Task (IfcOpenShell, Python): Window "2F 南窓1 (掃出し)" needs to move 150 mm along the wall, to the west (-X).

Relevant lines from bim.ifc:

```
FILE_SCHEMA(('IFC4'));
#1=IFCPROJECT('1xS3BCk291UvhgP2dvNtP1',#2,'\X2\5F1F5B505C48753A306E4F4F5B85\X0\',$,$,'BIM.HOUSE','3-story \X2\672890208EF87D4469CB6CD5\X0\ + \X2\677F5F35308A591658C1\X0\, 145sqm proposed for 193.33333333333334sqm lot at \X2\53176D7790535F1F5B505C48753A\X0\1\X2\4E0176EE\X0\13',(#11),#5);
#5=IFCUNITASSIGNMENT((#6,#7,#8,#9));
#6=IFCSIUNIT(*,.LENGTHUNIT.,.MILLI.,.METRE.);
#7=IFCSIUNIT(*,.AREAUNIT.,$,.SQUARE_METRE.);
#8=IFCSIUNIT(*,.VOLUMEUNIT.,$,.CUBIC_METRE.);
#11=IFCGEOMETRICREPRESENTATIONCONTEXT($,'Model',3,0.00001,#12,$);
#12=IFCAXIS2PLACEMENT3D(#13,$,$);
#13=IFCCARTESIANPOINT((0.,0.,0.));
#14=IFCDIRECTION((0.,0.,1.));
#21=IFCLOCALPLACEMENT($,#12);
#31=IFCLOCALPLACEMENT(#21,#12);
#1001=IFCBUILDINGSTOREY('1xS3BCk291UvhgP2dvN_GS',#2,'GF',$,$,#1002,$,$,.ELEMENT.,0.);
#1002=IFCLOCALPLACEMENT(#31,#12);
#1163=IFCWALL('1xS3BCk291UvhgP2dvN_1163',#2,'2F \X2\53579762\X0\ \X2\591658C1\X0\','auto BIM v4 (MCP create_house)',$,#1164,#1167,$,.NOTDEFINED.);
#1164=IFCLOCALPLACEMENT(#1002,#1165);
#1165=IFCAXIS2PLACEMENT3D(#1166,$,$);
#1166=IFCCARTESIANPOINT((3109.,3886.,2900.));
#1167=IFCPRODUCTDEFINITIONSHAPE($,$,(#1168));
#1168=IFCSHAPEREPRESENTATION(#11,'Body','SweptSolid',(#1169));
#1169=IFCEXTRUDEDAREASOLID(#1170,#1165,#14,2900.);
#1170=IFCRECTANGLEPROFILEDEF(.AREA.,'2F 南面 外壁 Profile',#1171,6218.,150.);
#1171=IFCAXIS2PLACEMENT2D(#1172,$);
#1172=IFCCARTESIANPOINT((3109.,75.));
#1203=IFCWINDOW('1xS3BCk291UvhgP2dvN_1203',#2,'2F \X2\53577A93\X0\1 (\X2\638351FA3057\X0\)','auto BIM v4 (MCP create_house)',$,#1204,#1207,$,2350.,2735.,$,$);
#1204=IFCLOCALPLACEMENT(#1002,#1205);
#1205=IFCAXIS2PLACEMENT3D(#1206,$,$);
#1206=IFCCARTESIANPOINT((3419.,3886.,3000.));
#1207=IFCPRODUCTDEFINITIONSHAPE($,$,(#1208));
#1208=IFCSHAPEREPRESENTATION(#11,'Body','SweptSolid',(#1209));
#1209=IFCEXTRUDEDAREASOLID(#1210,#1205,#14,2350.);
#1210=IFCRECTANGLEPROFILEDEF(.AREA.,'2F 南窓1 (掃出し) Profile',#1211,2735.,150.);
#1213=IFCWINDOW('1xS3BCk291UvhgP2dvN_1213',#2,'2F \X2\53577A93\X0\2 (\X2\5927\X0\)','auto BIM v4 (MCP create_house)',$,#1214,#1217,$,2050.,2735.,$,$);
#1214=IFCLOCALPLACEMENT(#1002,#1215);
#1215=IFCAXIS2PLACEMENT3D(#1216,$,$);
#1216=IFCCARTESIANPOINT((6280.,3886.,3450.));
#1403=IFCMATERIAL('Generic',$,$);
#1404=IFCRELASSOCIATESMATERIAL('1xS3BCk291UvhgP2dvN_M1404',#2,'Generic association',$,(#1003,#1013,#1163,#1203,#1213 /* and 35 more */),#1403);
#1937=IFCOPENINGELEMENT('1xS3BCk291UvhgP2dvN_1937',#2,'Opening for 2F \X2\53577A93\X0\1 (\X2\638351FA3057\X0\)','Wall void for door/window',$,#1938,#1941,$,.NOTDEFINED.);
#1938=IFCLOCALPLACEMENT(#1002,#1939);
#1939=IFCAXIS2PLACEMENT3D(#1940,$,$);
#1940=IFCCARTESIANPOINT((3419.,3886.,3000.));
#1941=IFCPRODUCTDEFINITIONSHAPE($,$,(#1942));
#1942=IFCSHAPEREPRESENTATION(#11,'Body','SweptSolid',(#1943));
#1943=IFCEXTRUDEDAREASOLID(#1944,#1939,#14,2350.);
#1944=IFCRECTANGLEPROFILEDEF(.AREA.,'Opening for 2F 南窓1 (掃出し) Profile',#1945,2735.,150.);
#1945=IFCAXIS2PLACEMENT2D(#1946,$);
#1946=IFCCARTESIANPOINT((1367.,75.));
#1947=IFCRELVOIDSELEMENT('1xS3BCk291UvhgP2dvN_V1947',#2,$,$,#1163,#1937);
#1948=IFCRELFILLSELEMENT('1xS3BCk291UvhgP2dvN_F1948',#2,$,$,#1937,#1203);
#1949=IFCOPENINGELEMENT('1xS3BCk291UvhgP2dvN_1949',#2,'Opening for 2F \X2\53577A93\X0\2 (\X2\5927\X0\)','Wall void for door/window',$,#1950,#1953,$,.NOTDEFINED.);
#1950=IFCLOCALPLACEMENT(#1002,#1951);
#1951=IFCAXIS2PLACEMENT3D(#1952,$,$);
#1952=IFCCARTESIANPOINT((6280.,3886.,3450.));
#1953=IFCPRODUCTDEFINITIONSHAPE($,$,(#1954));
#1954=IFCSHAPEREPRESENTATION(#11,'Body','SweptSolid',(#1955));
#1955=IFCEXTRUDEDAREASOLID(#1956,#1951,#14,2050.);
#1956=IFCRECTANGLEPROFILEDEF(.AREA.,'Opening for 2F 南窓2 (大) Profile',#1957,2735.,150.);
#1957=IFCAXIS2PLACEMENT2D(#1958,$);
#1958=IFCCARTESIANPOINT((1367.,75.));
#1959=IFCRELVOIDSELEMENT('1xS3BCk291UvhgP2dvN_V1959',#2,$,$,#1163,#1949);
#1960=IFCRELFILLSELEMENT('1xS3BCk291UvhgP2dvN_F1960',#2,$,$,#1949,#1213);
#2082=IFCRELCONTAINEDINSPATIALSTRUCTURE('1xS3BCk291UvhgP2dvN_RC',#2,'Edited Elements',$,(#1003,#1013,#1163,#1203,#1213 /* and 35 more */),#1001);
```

```python
import ifcopenshell
import ifcopenshell.api.geometry
import ifcopenshell.util.placement

model = ifcopenshell.open("bim.ifc")

window = model.by_guid("1xS3BCk291UvhgP2dvN_1203")
opening = window.FillsVoids[0].RelatingOpeningElement
wall = opening.VoidsElements[0].RelatingBuildingElement

wall_matrix = ifcopenshell.util.placement.get_local_placement(wall.ObjectPlacement)
shift = wall_matrix[:3, 0] * -150.0
before = ifcopenshell.util.placement.get_local_placement(window.ObjectPlacement)[:3, 3].copy()

# The window is not placed relative to its opening, so move both.
for product in (opening, window):
    matrix = ifcopenshell.util.placement.get_local_placement(product.ObjectPlacement)
    matrix[:3, 3] += shift
    ifcopenshell.api.geometry.edit_object_placement(model, product=product, matrix=matrix, is_si=False)

after = ifcopenshell.util.placement.get_local_placement(window.ObjectPlacement)[:3, 3]
print("window moved by", (after - before).round(3) + 0.0)

model.write("bim-out.ifc")
```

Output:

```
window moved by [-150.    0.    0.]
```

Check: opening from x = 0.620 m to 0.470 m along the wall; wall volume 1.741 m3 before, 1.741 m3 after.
